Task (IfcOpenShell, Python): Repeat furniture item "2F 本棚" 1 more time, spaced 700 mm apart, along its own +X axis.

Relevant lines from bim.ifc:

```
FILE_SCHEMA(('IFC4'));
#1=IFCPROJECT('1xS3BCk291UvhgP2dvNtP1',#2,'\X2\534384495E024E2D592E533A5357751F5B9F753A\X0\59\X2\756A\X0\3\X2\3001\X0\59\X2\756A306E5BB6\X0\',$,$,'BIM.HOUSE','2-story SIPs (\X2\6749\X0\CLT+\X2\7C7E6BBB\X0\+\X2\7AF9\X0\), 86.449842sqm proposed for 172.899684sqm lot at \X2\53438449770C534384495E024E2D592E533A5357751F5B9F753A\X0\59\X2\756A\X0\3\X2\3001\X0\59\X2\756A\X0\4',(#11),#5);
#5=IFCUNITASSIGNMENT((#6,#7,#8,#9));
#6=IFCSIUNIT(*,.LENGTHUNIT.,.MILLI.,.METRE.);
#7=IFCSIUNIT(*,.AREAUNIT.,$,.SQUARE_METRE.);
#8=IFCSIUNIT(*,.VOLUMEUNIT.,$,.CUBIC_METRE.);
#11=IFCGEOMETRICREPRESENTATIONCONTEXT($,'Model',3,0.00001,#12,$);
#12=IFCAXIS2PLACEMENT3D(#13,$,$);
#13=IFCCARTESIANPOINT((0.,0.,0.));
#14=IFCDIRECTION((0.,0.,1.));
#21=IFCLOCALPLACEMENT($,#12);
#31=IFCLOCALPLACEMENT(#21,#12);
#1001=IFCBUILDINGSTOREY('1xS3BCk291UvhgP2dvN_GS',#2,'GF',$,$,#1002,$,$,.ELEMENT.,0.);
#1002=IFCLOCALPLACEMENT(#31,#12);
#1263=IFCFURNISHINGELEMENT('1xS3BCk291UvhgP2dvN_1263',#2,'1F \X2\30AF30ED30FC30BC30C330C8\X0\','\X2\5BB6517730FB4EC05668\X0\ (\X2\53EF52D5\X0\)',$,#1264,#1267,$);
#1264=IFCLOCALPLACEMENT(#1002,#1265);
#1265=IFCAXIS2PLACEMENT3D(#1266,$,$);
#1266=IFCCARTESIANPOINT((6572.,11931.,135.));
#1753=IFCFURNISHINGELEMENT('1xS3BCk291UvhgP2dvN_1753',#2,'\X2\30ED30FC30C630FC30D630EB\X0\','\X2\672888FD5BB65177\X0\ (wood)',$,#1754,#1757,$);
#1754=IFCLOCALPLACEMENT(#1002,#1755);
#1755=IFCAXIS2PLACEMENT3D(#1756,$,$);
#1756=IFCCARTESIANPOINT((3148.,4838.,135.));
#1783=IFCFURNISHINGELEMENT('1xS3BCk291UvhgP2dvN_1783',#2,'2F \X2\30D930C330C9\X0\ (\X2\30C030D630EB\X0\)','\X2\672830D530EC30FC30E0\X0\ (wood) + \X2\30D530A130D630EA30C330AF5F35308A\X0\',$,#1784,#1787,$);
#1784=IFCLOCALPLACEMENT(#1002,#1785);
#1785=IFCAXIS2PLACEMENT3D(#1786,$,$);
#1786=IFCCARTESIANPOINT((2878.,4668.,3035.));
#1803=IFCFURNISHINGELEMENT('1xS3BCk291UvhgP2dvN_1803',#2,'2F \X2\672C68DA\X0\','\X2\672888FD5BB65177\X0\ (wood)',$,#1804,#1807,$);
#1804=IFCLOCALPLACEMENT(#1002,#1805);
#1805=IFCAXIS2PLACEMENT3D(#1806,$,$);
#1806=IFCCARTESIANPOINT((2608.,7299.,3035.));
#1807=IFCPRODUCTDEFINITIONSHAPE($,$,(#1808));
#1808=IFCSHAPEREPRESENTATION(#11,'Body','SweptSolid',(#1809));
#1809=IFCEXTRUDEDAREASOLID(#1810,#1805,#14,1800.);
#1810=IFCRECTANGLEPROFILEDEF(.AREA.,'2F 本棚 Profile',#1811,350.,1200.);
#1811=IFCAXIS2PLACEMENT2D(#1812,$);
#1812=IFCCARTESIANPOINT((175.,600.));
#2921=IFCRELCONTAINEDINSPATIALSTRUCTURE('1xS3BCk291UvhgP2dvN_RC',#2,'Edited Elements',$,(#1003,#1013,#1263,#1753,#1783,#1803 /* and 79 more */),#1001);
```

```python
import ifcopenshell
import ifcopenshell.api.geometry
import ifcopenshell.api.root
import ifcopenshell.util.element
import ifcopenshell.util.placement

model = ifcopenshell.open("bim.ifc")


def reuse_history(source, copy):
    """copy_class also copies each property set's owner history, people and application; keep the originals."""
    for rel in copy.IsDefinedBy:
        if rel.is_a("IfcRelDefinesByProperties") and (history := rel.RelatingPropertyDefinition.OwnerHistory):
            rel.RelatingPropertyDefinition.OwnerHistory = source.OwnerHistory
            ifcopenshell.util.element.remove_deep2(model, history)


source = model.by_guid("1xS3BCk291UvhgP2dvN_1803")
base = ifcopenshell.util.placement.get_local_placement(source.ObjectPlacement)
step = base[:3, 0] * 700.0

for i in range(1, 2):
    copy = ifcopenshell.api.root.copy_class(model, product=source)
    copy.Representation = ifcopenshell.util.element.copy_deep(
        model, source.Representation, exclude=["IfcGeometricRepresentationContext", "IfcRepresentationMap"]
    )
    reuse_history(source, copy)
    matrix = base.copy()
    matrix[:3, 3] += i * step
    print("added at", matrix[:3, 3].round(3) + 0.0)
    ifcopenshell.api.geometry.edit_object_placement(model, product=copy, matrix=matrix, is_si=False)

model.write("bim-out.ifc")
```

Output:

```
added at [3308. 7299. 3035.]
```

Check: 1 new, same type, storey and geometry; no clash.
